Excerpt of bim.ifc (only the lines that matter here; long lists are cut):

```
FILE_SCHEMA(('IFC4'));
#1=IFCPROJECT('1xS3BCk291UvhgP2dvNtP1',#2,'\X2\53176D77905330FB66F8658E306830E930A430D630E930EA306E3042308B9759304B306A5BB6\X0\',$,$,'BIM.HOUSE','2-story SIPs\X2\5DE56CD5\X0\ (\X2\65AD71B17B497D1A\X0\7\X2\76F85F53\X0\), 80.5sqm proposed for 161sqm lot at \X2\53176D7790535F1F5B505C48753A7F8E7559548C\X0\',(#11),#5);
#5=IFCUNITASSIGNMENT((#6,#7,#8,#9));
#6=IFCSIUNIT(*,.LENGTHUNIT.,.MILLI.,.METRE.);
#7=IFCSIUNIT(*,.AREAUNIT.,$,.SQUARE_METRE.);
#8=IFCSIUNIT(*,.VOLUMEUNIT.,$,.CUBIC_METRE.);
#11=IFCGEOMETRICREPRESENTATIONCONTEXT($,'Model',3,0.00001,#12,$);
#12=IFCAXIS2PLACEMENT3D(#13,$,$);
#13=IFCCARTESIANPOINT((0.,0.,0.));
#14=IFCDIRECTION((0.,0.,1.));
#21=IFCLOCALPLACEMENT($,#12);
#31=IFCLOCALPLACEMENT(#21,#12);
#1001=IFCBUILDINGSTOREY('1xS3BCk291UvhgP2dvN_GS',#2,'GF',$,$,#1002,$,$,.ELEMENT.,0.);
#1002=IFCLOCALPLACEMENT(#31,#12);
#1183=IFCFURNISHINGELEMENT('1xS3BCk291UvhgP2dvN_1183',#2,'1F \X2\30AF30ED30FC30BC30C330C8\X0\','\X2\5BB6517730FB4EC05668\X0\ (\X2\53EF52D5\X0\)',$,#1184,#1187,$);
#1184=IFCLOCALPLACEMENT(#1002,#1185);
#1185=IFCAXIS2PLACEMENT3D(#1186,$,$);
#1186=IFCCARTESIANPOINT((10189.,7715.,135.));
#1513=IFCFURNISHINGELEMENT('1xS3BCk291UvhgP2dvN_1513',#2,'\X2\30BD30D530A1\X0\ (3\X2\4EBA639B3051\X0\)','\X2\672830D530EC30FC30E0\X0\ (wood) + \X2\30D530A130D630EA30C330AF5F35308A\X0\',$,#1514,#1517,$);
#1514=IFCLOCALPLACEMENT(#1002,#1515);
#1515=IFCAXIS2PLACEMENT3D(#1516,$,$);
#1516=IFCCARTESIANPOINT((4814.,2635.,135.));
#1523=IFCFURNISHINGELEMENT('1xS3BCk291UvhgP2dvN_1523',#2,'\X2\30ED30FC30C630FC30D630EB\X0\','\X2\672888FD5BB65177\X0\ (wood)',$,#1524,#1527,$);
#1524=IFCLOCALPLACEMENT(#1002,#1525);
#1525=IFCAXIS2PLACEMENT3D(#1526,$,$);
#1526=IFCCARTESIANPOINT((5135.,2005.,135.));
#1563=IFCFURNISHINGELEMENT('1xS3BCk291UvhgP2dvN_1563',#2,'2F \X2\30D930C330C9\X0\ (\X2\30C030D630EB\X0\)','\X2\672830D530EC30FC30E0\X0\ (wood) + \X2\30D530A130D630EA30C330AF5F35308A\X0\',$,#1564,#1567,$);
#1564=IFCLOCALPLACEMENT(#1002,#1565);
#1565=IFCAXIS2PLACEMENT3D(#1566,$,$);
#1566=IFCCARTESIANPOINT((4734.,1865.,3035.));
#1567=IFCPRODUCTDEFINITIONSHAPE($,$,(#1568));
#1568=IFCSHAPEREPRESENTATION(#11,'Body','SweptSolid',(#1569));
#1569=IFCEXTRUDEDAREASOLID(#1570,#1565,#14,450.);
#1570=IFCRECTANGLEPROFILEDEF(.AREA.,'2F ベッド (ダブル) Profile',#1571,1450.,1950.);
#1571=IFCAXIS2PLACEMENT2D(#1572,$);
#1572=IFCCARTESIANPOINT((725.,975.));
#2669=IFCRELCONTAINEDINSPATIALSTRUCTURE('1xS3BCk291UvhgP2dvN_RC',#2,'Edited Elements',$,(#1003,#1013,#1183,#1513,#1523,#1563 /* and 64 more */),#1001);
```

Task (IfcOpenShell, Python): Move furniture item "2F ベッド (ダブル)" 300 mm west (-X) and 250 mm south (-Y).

```python
import ifcopenshell
import ifcopenshell.api.geometry
import ifcopenshell.util.placement
import ifcopenshell.util.unit

model = ifcopenshell.open("bim.ifc")
unit_scale = ifcopenshell.util.unit.calculate_unit_scale(model)

item = model.by_guid("1xS3BCk291UvhgP2dvN_1563")
matrix = ifcopenshell.util.placement.get_local_placement(item.ObjectPlacement)
matrix[0, 3] -= 0.3 / unit_scale
matrix[1, 3] -= 0.25 / unit_scale
ifcopenshell.api.geometry.edit_object_placement(model, product=item, matrix=matrix, is_si=False)

print(ifcopenshell.util.placement.get_local_placement(item.ObjectPlacement).round(3) + 0.0)

model.write("bim-out.ifc")
```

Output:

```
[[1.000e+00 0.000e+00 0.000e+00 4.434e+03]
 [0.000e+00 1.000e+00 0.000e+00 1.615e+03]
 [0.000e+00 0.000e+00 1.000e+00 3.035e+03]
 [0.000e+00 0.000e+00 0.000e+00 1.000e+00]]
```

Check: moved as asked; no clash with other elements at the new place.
